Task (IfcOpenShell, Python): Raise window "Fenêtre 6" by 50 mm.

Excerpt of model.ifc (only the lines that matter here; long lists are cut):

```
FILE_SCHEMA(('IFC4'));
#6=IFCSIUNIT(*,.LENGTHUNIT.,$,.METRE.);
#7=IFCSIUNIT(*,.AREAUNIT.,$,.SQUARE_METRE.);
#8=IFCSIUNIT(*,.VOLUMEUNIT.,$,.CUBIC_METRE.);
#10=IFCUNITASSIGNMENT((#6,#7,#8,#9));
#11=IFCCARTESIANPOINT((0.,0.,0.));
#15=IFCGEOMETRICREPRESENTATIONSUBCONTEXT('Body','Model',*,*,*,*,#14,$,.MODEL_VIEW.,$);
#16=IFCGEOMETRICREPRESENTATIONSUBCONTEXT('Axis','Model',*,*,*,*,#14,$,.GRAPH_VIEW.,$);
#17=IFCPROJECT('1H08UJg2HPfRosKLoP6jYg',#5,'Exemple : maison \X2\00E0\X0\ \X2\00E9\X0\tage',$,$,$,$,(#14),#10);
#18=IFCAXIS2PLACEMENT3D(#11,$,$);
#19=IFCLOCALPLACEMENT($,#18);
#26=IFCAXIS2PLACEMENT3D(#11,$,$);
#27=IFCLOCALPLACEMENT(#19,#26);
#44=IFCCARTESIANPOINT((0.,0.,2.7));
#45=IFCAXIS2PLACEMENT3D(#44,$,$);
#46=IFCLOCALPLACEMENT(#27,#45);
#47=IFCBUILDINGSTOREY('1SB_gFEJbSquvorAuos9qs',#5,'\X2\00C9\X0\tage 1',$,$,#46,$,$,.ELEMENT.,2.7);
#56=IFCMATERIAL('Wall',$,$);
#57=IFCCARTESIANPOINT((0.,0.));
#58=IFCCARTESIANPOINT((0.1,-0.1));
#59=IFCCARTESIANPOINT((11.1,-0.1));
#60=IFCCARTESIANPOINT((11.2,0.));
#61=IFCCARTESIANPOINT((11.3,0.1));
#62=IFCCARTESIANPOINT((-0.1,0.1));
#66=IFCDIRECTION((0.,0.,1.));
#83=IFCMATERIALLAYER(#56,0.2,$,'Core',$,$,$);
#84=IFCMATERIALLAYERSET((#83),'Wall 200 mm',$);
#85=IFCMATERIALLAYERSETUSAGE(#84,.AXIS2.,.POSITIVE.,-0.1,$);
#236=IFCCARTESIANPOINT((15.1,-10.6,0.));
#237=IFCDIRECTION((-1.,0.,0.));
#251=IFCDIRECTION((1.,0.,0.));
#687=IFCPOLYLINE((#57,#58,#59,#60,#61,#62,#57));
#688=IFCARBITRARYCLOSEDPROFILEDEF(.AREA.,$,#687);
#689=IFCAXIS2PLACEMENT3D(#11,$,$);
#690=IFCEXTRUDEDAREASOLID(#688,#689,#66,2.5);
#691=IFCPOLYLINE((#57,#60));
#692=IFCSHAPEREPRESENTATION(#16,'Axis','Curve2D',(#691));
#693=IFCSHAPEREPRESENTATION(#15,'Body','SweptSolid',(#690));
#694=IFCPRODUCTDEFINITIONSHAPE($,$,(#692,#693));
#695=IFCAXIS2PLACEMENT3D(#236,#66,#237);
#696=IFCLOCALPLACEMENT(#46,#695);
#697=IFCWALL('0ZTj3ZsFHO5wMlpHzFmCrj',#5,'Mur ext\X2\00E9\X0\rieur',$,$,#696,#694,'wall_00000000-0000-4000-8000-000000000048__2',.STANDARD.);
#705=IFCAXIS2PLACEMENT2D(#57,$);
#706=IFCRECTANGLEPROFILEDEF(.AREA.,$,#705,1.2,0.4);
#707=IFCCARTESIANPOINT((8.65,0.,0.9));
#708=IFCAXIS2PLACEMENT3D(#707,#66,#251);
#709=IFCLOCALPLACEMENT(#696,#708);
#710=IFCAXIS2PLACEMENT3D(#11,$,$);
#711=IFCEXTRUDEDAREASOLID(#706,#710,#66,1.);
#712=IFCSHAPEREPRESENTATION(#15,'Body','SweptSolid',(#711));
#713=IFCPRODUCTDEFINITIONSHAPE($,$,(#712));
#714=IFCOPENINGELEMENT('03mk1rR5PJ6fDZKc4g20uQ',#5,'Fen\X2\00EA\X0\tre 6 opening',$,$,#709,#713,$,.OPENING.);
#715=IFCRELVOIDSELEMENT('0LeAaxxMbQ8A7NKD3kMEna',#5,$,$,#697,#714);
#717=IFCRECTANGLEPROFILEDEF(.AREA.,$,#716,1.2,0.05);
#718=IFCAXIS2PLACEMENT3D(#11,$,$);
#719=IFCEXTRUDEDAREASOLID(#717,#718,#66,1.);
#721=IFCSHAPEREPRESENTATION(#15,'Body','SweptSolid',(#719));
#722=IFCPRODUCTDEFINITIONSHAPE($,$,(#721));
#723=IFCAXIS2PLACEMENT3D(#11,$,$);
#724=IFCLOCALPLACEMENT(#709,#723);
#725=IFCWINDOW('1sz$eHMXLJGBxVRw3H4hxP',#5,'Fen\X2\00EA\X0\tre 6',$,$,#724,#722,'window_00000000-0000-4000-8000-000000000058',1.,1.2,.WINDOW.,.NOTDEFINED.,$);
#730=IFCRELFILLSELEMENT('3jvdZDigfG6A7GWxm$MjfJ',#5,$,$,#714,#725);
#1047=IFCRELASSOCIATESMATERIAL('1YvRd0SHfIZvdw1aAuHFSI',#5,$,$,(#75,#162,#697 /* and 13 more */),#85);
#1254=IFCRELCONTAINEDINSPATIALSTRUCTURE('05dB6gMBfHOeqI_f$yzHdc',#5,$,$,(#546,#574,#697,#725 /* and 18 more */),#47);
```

```python
import numpy as np
import ifcopenshell
import ifcopenshell.api.geometry
import ifcopenshell.util.placement
import ifcopenshell.util.unit

model = ifcopenshell.open("model.ifc")
unit_scale = ifcopenshell.util.unit.calculate_unit_scale(model)

window = model.by_guid("1sz$eHMXLJGBxVRw3H4hxP")
opening = window.FillsVoids[0].RelatingOpeningElement
dz = 0.05

shift = np.array([0.0, 0.0, dz])
# The window is placed relative to its opening, so it follows when the opening moves.
matrix = ifcopenshell.util.placement.get_local_placement(opening.ObjectPlacement)
matrix[:3, 3] += shift
ifcopenshell.api.geometry.edit_object_placement(
    model, product=opening, matrix=matrix, is_si=False, should_transform_children=True
)

print(f"moved by {dz * unit_scale:+.3f} m")

model.write("model_edited.ifc")
```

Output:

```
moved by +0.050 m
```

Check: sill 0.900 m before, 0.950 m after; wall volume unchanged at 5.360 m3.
